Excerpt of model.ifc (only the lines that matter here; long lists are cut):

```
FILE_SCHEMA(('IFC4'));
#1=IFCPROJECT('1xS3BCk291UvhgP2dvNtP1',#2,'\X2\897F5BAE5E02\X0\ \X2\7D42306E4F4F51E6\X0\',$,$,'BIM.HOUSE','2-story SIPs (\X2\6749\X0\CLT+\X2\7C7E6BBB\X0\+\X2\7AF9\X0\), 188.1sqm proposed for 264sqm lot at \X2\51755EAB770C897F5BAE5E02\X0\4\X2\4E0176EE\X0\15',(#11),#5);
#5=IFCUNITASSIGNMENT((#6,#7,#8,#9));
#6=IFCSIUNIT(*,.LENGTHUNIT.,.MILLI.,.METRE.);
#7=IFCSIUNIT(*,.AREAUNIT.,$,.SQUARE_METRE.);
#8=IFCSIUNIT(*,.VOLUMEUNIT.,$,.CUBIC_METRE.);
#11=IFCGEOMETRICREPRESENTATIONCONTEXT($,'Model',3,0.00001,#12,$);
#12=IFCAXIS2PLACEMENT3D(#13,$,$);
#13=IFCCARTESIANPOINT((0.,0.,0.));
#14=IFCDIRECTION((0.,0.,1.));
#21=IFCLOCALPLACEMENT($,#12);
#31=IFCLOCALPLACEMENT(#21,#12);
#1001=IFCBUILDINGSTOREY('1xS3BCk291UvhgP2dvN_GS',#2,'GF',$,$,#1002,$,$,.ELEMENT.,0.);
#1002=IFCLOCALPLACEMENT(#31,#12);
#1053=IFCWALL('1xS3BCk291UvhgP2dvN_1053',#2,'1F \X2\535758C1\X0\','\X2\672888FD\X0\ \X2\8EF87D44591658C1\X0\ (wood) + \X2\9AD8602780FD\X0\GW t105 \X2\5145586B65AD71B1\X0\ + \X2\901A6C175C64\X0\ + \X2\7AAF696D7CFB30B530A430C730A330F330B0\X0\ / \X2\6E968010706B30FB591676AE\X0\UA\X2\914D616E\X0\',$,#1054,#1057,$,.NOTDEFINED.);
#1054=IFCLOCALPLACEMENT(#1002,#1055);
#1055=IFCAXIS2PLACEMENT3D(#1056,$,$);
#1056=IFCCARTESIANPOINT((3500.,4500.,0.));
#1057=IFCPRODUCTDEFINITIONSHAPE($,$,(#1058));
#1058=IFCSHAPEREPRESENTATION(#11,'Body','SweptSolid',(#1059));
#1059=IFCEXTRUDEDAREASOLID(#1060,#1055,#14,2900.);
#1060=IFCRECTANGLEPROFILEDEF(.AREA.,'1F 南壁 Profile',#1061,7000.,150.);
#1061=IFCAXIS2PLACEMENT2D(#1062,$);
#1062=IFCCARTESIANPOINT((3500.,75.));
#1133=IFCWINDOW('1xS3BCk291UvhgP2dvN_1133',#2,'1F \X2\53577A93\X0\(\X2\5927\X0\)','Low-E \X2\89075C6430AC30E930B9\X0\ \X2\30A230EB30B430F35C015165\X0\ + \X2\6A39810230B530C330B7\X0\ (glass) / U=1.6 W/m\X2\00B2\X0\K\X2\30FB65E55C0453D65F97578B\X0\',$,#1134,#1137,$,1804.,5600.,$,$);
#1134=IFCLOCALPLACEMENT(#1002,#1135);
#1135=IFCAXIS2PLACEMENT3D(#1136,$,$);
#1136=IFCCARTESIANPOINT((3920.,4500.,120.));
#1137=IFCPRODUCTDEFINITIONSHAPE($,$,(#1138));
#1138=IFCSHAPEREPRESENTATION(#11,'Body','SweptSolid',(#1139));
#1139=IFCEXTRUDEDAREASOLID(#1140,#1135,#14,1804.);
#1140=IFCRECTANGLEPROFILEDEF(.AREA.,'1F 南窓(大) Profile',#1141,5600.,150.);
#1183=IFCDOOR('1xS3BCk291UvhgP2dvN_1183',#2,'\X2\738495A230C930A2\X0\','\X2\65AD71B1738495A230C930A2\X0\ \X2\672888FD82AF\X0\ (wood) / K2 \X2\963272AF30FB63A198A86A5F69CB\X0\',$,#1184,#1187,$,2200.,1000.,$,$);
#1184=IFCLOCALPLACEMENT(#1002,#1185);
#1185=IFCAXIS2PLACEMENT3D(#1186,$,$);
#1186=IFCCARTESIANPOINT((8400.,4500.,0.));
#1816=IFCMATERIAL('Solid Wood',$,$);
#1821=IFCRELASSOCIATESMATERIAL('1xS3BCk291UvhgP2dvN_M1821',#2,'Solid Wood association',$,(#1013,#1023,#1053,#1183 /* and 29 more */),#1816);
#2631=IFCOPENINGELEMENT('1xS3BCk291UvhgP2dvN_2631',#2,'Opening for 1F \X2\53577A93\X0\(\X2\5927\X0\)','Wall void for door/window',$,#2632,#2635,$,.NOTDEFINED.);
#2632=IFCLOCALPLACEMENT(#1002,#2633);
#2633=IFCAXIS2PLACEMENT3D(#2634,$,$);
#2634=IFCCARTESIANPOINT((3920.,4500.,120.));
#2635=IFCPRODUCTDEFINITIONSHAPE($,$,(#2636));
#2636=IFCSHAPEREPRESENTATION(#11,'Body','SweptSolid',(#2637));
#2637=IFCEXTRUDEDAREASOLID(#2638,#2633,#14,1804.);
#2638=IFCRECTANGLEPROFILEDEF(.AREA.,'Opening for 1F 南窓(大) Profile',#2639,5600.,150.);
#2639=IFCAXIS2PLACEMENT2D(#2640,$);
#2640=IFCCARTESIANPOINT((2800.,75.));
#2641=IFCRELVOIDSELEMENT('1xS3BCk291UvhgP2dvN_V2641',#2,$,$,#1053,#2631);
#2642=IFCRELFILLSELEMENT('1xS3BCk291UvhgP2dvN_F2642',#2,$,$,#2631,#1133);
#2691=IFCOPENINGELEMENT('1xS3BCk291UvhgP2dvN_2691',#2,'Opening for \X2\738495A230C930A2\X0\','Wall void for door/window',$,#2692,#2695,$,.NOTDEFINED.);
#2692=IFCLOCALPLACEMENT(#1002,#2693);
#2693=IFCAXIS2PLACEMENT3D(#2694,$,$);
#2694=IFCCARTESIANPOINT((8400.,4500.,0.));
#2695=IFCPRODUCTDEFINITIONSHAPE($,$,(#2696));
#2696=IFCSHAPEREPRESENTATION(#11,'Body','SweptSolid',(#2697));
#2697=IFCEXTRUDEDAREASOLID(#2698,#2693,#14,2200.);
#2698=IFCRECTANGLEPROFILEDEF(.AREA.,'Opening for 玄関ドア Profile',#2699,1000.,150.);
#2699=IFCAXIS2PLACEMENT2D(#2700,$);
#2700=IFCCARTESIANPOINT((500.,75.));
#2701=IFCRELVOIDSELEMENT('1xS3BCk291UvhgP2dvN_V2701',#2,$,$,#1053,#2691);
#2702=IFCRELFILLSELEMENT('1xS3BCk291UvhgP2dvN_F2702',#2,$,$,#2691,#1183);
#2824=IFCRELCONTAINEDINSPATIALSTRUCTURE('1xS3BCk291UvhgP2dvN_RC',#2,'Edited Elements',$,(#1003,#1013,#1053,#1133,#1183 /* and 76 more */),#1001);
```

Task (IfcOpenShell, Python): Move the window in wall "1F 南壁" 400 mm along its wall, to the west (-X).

```python
import ifcopenshell
import ifcopenshell.api.geometry
import ifcopenshell.util.placement
import ifcopenshell.util.unit

model = ifcopenshell.open("model.ifc")
unit_scale = ifcopenshell.util.unit.calculate_unit_scale(model)

window = model.by_guid("1xS3BCk291UvhgP2dvN_1133")
opening = window.FillsVoids[0].RelatingOpeningElement
wall = opening.VoidsElements[0].RelatingBuildingElement

wall_matrix = ifcopenshell.util.placement.get_local_placement(wall.ObjectPlacement)
shift = wall_matrix[:3, 0] * -0.4 / unit_scale
before = ifcopenshell.util.placement.get_local_placement(window.ObjectPlacement)[:3, 3].copy()

# The window is not placed relative to its opening, so move both.
for product in (opening, window):
    matrix = ifcopenshell.util.placement.get_local_placement(product.ObjectPlacement)
    matrix[:3, 3] += shift
    ifcopenshell.api.geometry.edit_object_placement(model, product=product, matrix=matrix, is_si=False)

after = ifcopenshell.util.placement.get_local_placement(window.ObjectPlacement)[:3, 3]
print("window moved by", (after - before).round(3) + 0.0)

model.write("model_updated.ifc")
```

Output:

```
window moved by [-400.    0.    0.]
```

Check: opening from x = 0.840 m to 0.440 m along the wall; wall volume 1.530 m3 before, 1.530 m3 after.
